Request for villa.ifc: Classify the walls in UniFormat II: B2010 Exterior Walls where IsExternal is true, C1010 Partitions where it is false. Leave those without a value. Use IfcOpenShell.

First a look at what the model holds.

```python
import ifcopenshell
import ifcopenshell.util.element

model = ifcopenshell.open("villa.ifc")
print(model.schema)
print("classifications:", [c.Name for c in model.by_type("IfcClassification")])
values = [ifcopenshell.util.element.get_pset(e, "Pset_WallCommon", "IsExternal") for e in model.by_type("IfcWall")]
for value in (True, False, None):
    print("IsExternal", value, values.count(value))
```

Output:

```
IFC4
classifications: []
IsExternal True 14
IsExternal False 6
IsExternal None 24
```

```python
import ifcopenshell
import ifcopenshell.api.classification
import ifcopenshell.util.element

model = ifcopenshell.open("villa.ifc")

system = ifcopenshell.api.classification.add_classification(model, classification="UniFormat II")

walls = model.by_type("IfcWall")
external = {e: ifcopenshell.util.element.get_pset(e, "Pset_WallCommon", "IsExternal") for e in walls}
for flag, code, name in ((True, "B2010", "Exterior Walls"), (False, "C1010", "Partitions")):
    products = [e for e in walls if external[e] is flag]
    ifcopenshell.api.classification.add_reference(
        model, products=products, classification=system, identification=code, name=name
    )
    print(code, len(products))

model.write("villa_rev.ifc")
```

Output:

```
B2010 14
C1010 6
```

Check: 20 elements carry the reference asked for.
